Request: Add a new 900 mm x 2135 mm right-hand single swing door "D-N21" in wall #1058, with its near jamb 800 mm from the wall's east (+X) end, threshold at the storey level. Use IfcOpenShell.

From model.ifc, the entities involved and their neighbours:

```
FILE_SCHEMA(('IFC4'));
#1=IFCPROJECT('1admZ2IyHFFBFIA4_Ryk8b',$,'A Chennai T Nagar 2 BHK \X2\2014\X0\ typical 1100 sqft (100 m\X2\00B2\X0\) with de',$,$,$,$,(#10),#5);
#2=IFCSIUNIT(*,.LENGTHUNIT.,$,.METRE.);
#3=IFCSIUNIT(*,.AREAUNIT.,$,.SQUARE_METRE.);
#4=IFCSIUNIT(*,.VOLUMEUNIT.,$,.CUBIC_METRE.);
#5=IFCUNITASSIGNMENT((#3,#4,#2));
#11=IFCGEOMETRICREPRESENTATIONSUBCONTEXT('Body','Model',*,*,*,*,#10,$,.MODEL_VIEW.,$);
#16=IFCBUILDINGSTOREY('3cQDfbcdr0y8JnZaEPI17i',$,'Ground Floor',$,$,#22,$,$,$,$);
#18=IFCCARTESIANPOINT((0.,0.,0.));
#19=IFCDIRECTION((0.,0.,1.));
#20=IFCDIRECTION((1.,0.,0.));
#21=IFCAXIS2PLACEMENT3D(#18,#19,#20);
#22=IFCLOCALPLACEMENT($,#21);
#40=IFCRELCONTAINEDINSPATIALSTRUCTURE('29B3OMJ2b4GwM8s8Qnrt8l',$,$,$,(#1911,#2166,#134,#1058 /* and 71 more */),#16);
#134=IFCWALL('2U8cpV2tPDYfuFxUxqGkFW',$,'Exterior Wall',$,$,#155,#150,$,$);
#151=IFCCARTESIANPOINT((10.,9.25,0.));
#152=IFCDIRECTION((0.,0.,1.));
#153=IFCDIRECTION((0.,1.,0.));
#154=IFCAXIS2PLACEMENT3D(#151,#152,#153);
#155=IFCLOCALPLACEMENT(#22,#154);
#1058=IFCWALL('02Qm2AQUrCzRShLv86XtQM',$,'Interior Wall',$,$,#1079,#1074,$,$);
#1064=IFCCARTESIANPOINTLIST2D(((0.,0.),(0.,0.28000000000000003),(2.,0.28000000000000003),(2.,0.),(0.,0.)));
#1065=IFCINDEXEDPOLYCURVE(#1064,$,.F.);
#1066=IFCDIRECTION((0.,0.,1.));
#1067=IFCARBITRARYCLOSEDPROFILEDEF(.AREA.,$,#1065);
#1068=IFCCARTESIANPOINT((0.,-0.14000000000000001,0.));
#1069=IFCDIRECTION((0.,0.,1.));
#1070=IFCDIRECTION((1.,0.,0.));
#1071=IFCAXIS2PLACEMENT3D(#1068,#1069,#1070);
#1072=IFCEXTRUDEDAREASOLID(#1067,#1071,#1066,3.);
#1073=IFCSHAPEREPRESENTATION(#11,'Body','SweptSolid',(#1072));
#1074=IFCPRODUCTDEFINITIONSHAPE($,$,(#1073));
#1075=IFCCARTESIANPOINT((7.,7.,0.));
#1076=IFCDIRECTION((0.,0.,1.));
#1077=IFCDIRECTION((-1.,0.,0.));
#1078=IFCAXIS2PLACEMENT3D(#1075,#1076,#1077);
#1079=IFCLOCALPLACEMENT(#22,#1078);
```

```python
import numpy as np
import ifcopenshell
import ifcopenshell.api.feature
import ifcopenshell.api.geometry
import ifcopenshell.api.root
import ifcopenshell.api.spatial
import ifcopenshell.geom
import ifcopenshell.util.element
import ifcopenshell.util.placement
import ifcopenshell.util.representation
import ifcopenshell.util.shape
import ifcopenshell.util.unit

model = ifcopenshell.open("model.ifc")
unit_scale = ifcopenshell.util.unit.calculate_unit_scale(model)
settings = ifcopenshell.geom.settings()


def volume(element):
    """Net volume in cubic metres, openings subtracted."""
    shape = ifcopenshell.geom.create_shape(settings, element)
    return ifcopenshell.util.shape.get_volume(shape.geometry)


wall = model.by_id(1058)
storey = ifcopenshell.util.element.get_container(wall, ifc_class="IfcBuildingStorey")
context = ifcopenshell.util.representation.get_context(model, "Model", "Body", "MODEL_VIEW")
before = volume(wall)

width, height, from_end, sill = 0.9, 2.135, 0.8, 0.0  # metres

# The wall runs along its own X axis, and the end named is its -X end.
wall_shape = ifcopenshell.geom.create_shape(settings, wall)
x, y, z = ifcopenshell.util.shape.get_vertices(wall_shape.geometry).T
start = x.min() + from_end
face, thickness = float(y.min()), float(y.max() - y.min())
wall_matrix = ifcopenshell.util.placement.get_local_placement(wall.ObjectPlacement)
level = ifcopenshell.util.placement.get_local_placement(storey.ObjectPlacement)[2, 3]


def in_wall(x, y):
    """Placement at x, y metres in the wall's axes, at sill height."""
    matrix = wall_matrix.copy()
    matrix[:, 3] = wall_matrix @ np.array([x / unit_scale, y / unit_scale, 0.0, 1.0])
    matrix[2, 3] = level + sill / unit_scale
    return matrix


# Opening: a box that overshoots both wall faces by 50 mm.
opening = ifcopenshell.api.root.create_entity(model, ifc_class="IfcOpeningElement", predefined_type="OPENING")
box = ifcopenshell.api.geometry.add_wall_representation(
    model, context=context, length=width, height=height, thickness=thickness + 0.1
)
ifcopenshell.api.geometry.assign_representation(model, product=opening, representation=box)
ifcopenshell.api.geometry.edit_object_placement(model, product=opening, matrix=in_wall(start, face - 0.05), is_si=False)
ifcopenshell.api.feature.add_feature(model, feature=opening, element=wall)

door = ifcopenshell.api.root.create_entity(model, ifc_class="IfcDoor", name="D-N21", predefined_type="DOOR")
door.OverallWidth, door.OverallHeight = width / unit_scale, height / unit_scale
door.OperationType = "SINGLE_SWING_RIGHT"
body = ifcopenshell.api.geometry.add_door_representation(
    model,
    context=context,
    overall_width=door.OverallWidth,
    overall_height=door.OverallHeight,
    operation_type="SINGLE_SWING_RIGHT",
    lining_properties={"LiningDepth": thickness / unit_scale, "ThresholdDepth": thickness / unit_scale},
)
ifcopenshell.api.geometry.assign_representation(model, product=door, representation=body)
ifcopenshell.api.spatial.assign_container(model, products=[door], relating_structure=storey)
ifcopenshell.api.feature.add_filling(model, opening=opening, element=door)

# The lining spans the wall, so the door starts at the wall face.
ifcopenshell.api.geometry.edit_object_placement(model, product=door, matrix=in_wall(start, face), is_si=False)

after = volume(wall)

print(f"wall volume {before:.3f} -> {after:.3f} m3")

model.write("model_updated.ifc")
```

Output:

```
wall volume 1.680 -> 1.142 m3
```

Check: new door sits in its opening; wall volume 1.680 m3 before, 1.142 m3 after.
